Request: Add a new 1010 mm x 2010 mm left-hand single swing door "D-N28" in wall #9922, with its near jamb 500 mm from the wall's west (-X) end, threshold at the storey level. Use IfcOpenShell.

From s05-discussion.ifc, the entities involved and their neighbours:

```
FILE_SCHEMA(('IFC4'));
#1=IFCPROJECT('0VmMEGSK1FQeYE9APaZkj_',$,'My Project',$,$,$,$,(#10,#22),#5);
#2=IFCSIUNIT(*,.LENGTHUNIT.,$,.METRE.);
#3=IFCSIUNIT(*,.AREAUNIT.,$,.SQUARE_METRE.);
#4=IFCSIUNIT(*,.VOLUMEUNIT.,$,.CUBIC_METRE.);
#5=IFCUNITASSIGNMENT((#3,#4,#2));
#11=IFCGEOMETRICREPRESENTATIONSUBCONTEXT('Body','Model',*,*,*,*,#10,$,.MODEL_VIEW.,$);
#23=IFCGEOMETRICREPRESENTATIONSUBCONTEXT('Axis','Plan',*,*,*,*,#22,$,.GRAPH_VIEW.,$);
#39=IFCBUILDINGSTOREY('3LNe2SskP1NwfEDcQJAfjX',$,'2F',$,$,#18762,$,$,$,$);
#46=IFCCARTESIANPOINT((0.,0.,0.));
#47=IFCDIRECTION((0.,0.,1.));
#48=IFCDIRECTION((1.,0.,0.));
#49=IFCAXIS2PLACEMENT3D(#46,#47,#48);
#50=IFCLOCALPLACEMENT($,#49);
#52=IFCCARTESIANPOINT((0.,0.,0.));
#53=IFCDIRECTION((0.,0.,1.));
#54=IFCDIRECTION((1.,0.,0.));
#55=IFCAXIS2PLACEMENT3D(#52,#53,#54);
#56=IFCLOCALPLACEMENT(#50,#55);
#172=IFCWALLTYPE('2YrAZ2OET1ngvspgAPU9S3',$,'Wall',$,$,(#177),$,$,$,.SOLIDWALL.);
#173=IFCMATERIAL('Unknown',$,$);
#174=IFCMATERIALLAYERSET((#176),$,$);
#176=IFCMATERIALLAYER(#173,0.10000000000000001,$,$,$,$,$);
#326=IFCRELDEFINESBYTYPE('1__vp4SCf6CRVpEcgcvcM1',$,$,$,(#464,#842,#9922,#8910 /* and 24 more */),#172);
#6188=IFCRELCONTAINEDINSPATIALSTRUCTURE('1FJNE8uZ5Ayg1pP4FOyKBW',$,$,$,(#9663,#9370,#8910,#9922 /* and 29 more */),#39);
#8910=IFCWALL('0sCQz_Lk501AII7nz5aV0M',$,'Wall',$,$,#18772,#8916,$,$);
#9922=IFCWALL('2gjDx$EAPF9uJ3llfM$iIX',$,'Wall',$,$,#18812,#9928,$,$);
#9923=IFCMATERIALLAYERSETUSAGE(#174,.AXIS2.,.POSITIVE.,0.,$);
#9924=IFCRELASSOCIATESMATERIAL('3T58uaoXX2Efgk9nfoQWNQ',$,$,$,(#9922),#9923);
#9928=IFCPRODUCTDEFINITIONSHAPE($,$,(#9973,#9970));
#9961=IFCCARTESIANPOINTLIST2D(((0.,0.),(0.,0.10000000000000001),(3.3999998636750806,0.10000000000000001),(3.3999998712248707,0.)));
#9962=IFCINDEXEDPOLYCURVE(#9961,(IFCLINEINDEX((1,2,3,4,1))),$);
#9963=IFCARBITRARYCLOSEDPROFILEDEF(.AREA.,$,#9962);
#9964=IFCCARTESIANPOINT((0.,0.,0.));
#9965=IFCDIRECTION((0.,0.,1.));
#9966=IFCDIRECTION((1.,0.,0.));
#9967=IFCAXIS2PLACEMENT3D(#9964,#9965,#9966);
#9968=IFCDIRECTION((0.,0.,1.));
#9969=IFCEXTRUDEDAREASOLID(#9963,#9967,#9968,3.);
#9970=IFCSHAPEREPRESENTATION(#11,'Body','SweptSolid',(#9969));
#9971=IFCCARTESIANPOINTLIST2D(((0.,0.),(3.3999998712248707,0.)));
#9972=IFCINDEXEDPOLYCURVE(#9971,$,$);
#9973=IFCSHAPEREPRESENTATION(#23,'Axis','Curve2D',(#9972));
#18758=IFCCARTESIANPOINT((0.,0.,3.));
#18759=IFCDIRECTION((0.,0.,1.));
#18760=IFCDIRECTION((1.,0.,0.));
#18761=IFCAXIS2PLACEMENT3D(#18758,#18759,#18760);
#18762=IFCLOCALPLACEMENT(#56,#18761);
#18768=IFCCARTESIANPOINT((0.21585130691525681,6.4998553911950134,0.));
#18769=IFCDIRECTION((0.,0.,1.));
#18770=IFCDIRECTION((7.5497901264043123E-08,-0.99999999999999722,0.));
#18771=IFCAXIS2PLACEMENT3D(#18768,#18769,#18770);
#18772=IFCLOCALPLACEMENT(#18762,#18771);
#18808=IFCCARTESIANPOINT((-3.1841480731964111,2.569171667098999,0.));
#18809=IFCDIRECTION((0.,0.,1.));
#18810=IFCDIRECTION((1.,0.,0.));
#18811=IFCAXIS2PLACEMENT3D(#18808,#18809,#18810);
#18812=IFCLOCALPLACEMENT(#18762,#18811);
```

```python
import numpy as np
import ifcopenshell
import ifcopenshell.api.feature
import ifcopenshell.api.geometry
import ifcopenshell.api.root
import ifcopenshell.api.spatial
import ifcopenshell.geom
import ifcopenshell.util.element
import ifcopenshell.util.placement
import ifcopenshell.util.representation
import ifcopenshell.util.shape
import ifcopenshell.util.unit

model = ifcopenshell.open("s05-discussion.ifc")
unit_scale = ifcopenshell.util.unit.calculate_unit_scale(model)
settings = ifcopenshell.geom.settings()


def volume(element):
    """Net volume in cubic metres, openings subtracted."""
    shape = ifcopenshell.geom.create_shape(settings, element)
    return ifcopenshell.util.shape.get_volume(shape.geometry)


wall = model.by_guid("2gjDx$EAPF9uJ3llfM$iIX")
storey = ifcopenshell.util.element.get_container(wall, ifc_class="IfcBuildingStorey")
context = ifcopenshell.util.representation.get_context(model, "Model", "Body", "MODEL_VIEW")
before = volume(wall)

width, height, from_end, sill = 1.01, 2.01, 0.5, 0.0  # metres

# The wall runs along its own X axis, and the end named is its -X end.
wall_shape = ifcopenshell.geom.create_shape(settings, wall)
x, y, z = ifcopenshell.util.shape.get_vertices(wall_shape.geometry).T
start = x.min() + from_end
face, thickness = float(y.min()), float(y.max() - y.min())
wall_matrix = ifcopenshell.util.placement.get_local_placement(wall.ObjectPlacement)
level = ifcopenshell.util.placement.get_local_placement(storey.ObjectPlacement)[2, 3]


def in_wall(x, y):
    """Placement at x, y metres in the wall's axes, at sill height."""
    matrix = wall_matrix.copy()
    matrix[:, 3] = wall_matrix @ np.array([x / unit_scale, y / unit_scale, 0.0, 1.0])
    matrix[2, 3] = level + sill / unit_scale
    return matrix


# Opening: a box that overshoots both wall faces by 50 mm.
opening = ifcopenshell.api.root.create_entity(model, ifc_class="IfcOpeningElement", predefined_type="OPENING")
box = ifcopenshell.api.geometry.add_wall_representation(
    model, context=context, length=width, height=height, thickness=thickness + 0.1
)
ifcopenshell.api.geometry.assign_representation(model, product=opening, representation=box)
ifcopenshell.api.geometry.edit_object_placement(model, product=opening, matrix=in_wall(start, face - 0.05), is_si=False)
ifcopenshell.api.feature.add_feature(model, feature=opening, element=wall)

door = ifcopenshell.api.root.create_entity(model, ifc_class="IfcDoor", name="D-N28", predefined_type="DOOR")
door.OverallWidth, door.OverallHeight = width / unit_scale, height / unit_scale
door.OperationType = "SINGLE_SWING_LEFT"
body = ifcopenshell.api.geometry.add_door_representation(
    model,
    context=context,
    overall_width=door.OverallWidth,
    overall_height=door.OverallHeight,
    operation_type="SINGLE_SWING_LEFT",
    lining_properties={"LiningDepth": thickness / unit_scale, "ThresholdDepth": thickness / unit_scale},
)
ifcopenshell.api.geometry.assign_representation(model, product=door, representation=body)
ifcopenshell.api.spatial.assign_container(model, products=[door], relating_structure=storey)
ifcopenshell.api.feature.add_filling(model, opening=opening, element=door)

# The lining spans the wall, so the door starts at the wall face.
ifcopenshell.api.geometry.edit_object_placement(model, product=door, matrix=in_wall(start, face), is_si=False)

after = volume(wall)

print(f"wall volume {before:.3f} -> {after:.3f} m3")

model.write("s05-discussion_v2.ifc")
```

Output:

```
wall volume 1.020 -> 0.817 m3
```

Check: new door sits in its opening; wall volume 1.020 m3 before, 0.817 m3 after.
